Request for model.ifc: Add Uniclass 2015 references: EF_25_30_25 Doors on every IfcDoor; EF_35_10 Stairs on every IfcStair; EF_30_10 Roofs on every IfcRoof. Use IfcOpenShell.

First a look at what the model holds.

```python
import ifcopenshell

model = ifcopenshell.open("model.ifc")
print(model.schema)
print("classifications:", [c.Name for c in model.by_type("IfcClassification")])
for ifc_class in ("IfcDoor", "IfcRoof", "IfcStair", "IfcWall", "IfcWindow"):
    print(ifc_class, len(model.by_type(ifc_class)))
```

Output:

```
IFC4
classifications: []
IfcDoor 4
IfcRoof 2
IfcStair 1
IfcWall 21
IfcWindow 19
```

```python
import ifcopenshell
import ifcopenshell.api.classification

model = ifcopenshell.open("model.ifc")

system = ifcopenshell.api.classification.add_classification(model, classification="Uniclass 2015")

codes = {
    "IfcDoor": ("EF_25_30_25", "Doors"),
    "IfcStair": ("EF_35_10", "Stairs"),
    "IfcRoof": ("EF_30_10", "Roofs"),
}
for ifc_class, (code, name) in codes.items():
    products = model.by_type(ifc_class)
    ifcopenshell.api.classification.add_reference(
        model, products=products, classification=system, identification=code, name=name
    )
    print(code, len(products))

model.write("model-out.ifc")
```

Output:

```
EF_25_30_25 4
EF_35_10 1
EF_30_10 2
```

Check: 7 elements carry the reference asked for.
